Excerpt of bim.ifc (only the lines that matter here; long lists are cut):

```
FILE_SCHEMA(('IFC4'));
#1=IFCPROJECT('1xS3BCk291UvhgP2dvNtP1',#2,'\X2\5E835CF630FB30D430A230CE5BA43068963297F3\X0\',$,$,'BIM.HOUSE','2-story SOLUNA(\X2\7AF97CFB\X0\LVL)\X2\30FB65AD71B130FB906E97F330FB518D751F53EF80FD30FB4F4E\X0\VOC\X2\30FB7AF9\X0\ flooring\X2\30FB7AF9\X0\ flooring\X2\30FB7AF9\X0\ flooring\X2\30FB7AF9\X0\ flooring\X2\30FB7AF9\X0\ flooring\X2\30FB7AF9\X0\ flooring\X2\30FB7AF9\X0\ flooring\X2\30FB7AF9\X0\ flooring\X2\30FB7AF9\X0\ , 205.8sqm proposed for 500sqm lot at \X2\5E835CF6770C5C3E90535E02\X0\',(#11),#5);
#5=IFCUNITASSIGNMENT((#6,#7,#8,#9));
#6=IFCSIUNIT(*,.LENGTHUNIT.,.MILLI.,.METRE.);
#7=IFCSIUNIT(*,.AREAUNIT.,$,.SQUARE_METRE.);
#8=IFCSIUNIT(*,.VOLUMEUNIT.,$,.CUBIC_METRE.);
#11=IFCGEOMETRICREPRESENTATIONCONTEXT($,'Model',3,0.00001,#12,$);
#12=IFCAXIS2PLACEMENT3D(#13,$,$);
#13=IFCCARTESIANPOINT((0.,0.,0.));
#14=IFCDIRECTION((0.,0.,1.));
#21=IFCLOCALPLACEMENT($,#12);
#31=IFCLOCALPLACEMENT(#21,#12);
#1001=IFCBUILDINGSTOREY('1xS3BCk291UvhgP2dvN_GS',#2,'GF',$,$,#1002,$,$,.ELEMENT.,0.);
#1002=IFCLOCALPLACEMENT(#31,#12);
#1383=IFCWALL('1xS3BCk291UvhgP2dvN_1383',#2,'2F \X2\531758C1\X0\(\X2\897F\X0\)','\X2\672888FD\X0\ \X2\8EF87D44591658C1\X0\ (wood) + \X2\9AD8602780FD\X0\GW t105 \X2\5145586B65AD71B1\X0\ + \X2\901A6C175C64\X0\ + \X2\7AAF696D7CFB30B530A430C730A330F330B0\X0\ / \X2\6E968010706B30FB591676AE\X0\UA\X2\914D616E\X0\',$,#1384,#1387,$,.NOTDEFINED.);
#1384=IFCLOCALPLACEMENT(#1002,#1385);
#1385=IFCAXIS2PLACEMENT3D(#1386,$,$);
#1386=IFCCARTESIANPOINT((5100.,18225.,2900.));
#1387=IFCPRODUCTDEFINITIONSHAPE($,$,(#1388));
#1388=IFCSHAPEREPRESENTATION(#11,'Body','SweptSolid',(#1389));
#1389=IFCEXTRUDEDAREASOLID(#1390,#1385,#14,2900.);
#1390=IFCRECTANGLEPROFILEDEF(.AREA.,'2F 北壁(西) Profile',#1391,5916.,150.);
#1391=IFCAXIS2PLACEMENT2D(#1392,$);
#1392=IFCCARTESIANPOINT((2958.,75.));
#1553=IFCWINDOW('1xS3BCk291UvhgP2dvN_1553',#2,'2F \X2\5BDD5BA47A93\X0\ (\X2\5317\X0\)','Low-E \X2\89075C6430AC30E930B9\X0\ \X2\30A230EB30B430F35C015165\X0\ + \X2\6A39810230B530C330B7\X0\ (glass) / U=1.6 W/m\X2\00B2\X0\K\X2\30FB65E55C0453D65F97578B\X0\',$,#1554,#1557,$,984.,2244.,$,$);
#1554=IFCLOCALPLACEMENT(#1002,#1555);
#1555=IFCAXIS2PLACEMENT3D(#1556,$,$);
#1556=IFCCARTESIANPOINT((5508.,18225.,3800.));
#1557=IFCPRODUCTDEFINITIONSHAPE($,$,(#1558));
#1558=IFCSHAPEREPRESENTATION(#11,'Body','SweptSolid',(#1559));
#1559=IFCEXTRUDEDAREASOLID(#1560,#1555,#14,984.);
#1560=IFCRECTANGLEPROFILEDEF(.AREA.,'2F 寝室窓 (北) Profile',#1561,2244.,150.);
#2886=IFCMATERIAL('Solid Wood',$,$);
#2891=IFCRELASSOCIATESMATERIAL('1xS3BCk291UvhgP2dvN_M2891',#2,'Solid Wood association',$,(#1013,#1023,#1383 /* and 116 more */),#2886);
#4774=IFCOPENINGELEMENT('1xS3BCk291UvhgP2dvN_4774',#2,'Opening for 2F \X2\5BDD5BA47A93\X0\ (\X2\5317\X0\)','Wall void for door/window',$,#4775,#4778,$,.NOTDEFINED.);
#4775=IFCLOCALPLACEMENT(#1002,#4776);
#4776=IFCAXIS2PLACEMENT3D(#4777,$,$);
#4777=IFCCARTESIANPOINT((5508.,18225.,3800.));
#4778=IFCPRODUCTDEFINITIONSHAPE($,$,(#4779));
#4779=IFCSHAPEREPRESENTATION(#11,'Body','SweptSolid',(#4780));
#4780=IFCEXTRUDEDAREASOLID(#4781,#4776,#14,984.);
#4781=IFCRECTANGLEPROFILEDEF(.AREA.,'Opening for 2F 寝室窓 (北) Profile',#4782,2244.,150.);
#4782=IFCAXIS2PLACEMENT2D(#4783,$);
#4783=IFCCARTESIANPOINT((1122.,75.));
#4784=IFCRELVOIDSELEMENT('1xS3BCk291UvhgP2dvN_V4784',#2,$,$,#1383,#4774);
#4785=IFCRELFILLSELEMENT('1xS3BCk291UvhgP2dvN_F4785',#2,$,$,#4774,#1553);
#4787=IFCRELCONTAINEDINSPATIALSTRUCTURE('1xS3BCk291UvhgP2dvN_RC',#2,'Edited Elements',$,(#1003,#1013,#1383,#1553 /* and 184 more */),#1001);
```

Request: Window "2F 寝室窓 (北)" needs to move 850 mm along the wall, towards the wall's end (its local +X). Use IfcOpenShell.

```python
import ifcopenshell
import ifcopenshell.api.geometry
import ifcopenshell.util.placement

model = ifcopenshell.open("bim.ifc")

window = model.by_guid("1xS3BCk291UvhgP2dvN_1553")
opening = window.FillsVoids[0].RelatingOpeningElement
wall = opening.VoidsElements[0].RelatingBuildingElement

wall_matrix = ifcopenshell.util.placement.get_local_placement(wall.ObjectPlacement)
shift = wall_matrix[:3, 0] * 850.0
before = ifcopenshell.util.placement.get_local_placement(window.ObjectPlacement)[:3, 3].copy()

# The window is not placed relative to its opening, so move both.
for product in (opening, window):
    matrix = ifcopenshell.util.placement.get_local_placement(product.ObjectPlacement)
    matrix[:3, 3] += shift
    ifcopenshell.api.geometry.edit_object_placement(model, product=product, matrix=matrix, is_si=False)

after = ifcopenshell.util.placement.get_local_placement(window.ObjectPlacement)[:3, 3]
print("window moved by", (after - before).round(3) + 0.0)

model.write("bim_v2.ifc")
```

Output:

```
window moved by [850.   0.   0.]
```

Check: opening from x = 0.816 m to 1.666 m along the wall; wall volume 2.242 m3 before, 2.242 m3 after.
